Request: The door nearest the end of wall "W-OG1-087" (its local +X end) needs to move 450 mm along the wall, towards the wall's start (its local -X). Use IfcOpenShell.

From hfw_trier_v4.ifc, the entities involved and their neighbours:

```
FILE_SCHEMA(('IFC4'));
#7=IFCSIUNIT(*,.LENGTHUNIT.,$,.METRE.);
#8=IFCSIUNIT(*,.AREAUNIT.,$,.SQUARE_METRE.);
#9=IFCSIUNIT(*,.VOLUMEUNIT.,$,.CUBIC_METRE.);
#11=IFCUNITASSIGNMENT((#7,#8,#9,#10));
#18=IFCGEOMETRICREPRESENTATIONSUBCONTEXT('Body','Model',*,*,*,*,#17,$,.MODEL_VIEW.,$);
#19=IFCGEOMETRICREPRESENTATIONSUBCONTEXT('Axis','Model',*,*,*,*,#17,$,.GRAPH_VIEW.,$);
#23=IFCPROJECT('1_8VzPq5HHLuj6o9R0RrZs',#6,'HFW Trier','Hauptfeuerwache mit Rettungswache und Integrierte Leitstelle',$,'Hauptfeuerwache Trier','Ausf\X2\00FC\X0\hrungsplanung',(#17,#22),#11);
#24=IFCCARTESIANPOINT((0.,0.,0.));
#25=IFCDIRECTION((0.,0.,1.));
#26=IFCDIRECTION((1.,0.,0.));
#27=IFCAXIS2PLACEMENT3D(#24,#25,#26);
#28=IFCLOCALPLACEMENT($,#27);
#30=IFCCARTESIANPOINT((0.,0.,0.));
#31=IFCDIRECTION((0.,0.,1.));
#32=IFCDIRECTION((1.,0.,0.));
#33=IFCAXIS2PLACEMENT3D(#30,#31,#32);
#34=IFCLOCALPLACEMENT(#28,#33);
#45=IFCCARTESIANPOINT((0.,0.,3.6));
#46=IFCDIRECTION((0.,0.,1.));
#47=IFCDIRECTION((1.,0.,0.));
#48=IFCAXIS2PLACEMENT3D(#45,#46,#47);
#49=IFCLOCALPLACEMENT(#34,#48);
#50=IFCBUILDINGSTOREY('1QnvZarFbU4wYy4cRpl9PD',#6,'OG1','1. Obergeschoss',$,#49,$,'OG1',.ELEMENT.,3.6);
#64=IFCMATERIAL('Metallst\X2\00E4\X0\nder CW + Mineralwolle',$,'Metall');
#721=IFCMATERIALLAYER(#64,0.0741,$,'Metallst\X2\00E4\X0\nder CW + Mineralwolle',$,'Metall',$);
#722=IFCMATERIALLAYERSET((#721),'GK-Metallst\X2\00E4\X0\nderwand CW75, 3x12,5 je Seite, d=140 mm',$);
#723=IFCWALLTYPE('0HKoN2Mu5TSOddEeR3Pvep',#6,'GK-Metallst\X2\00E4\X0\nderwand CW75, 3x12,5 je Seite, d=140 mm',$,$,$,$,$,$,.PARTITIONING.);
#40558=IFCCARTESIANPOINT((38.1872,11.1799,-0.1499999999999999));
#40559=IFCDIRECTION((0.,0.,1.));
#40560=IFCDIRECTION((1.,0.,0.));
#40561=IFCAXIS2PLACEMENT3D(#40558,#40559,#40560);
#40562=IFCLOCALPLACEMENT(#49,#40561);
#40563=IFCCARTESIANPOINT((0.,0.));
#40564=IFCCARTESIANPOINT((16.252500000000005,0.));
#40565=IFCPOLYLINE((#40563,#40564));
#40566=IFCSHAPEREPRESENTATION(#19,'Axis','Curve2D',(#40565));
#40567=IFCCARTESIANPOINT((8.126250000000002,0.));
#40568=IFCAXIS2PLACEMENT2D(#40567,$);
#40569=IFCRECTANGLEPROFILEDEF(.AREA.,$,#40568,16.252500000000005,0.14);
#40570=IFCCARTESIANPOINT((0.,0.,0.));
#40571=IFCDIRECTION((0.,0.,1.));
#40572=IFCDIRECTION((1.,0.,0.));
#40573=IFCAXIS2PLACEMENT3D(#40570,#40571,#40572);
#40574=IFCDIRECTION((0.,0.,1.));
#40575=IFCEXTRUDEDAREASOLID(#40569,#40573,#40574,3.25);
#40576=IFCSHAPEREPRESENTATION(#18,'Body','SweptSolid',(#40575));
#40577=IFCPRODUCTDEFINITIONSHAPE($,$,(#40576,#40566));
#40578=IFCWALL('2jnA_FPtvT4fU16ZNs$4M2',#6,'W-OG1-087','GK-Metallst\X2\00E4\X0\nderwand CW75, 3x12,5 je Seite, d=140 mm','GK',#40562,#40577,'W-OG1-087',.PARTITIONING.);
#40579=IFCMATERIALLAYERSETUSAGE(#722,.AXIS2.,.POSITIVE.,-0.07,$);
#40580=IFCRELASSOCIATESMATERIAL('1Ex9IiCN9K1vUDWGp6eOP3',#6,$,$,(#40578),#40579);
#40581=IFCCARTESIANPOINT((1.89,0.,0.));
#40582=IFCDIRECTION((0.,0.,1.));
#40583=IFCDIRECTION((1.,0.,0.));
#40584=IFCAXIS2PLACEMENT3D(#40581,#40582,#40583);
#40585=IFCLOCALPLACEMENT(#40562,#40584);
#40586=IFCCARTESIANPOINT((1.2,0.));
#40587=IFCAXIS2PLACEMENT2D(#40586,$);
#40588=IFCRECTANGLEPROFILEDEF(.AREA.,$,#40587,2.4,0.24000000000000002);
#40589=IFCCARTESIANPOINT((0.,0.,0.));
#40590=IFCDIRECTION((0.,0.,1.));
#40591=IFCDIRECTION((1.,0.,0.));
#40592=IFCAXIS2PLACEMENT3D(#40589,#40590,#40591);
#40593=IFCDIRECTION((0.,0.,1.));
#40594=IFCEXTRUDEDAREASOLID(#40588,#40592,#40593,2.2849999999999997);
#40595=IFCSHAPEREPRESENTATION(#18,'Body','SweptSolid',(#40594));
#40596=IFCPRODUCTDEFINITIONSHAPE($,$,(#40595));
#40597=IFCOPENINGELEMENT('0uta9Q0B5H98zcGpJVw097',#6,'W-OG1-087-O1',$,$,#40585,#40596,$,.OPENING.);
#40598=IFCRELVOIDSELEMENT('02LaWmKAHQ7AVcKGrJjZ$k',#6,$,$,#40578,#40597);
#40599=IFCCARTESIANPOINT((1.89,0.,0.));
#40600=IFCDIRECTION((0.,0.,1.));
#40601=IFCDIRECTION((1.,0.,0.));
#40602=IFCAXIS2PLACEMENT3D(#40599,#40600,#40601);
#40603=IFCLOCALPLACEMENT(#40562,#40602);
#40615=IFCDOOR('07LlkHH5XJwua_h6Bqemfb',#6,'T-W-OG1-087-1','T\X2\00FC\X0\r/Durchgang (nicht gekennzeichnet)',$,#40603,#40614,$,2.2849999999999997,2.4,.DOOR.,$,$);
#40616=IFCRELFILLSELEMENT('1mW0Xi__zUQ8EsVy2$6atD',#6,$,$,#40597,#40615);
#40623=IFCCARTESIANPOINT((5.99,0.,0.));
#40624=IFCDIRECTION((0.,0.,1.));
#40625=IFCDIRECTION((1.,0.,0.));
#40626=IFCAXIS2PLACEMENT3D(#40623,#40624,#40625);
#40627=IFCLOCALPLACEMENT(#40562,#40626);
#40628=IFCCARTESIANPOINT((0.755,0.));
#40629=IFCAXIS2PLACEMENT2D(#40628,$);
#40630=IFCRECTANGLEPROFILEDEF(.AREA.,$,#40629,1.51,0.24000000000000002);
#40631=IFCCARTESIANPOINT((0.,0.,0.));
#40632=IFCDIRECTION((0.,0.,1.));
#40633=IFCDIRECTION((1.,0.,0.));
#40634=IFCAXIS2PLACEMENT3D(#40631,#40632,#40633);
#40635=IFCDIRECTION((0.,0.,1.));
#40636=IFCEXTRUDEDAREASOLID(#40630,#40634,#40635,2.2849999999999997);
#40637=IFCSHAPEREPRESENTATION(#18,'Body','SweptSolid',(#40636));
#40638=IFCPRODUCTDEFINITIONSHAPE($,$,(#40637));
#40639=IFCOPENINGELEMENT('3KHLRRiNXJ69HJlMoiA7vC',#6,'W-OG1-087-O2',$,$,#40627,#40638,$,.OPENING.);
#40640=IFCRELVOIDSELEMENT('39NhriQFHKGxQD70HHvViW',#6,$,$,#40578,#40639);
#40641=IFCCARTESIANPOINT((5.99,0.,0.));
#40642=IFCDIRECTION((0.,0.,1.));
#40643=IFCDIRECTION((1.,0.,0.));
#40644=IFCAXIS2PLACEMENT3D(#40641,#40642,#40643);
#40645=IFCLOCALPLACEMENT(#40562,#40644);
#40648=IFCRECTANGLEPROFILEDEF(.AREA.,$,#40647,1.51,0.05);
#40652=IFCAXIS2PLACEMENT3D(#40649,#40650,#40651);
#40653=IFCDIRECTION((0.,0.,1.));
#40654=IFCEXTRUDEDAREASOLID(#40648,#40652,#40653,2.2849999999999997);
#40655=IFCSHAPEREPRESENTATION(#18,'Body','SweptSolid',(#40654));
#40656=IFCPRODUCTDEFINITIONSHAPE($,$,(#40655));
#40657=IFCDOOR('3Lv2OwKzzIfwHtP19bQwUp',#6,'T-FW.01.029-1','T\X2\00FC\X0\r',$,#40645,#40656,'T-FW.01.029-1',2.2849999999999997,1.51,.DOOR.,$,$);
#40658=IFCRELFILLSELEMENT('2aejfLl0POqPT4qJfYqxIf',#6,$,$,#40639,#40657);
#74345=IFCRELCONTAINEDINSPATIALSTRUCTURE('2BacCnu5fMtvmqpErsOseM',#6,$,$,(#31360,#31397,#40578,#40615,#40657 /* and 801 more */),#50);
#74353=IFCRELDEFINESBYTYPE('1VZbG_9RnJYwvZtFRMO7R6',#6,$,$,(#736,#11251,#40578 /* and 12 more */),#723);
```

```python
import ifcopenshell
import ifcopenshell.api.geometry
import ifcopenshell.util.placement
import ifcopenshell.util.unit

model = ifcopenshell.open("hfw_trier_v4.ifc")
unit_scale = ifcopenshell.util.unit.calculate_unit_scale(model)

door = model.by_id(40657)
opening = door.FillsVoids[0].RelatingOpeningElement
wall = opening.VoidsElements[0].RelatingBuildingElement

wall_matrix = ifcopenshell.util.placement.get_local_placement(wall.ObjectPlacement)
shift = wall_matrix[:3, 0] * -0.45 / unit_scale
before = ifcopenshell.util.placement.get_local_placement(door.ObjectPlacement)[:3, 3].copy()

# The door is not placed relative to its opening, so move both.
for product in (opening, door):
    matrix = ifcopenshell.util.placement.get_local_placement(product.ObjectPlacement)
    matrix[:3, 3] += shift
    ifcopenshell.api.geometry.edit_object_placement(model, product=product, matrix=matrix, is_si=False)

after = ifcopenshell.util.placement.get_local_placement(door.ObjectPlacement)[:3, 3]
print("door moved by", (after - before).round(3) + 0.0)

model.write("hfw_trier_v4_rev.ifc")
```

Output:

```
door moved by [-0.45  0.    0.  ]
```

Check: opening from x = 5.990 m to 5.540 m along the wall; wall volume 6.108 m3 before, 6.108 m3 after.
